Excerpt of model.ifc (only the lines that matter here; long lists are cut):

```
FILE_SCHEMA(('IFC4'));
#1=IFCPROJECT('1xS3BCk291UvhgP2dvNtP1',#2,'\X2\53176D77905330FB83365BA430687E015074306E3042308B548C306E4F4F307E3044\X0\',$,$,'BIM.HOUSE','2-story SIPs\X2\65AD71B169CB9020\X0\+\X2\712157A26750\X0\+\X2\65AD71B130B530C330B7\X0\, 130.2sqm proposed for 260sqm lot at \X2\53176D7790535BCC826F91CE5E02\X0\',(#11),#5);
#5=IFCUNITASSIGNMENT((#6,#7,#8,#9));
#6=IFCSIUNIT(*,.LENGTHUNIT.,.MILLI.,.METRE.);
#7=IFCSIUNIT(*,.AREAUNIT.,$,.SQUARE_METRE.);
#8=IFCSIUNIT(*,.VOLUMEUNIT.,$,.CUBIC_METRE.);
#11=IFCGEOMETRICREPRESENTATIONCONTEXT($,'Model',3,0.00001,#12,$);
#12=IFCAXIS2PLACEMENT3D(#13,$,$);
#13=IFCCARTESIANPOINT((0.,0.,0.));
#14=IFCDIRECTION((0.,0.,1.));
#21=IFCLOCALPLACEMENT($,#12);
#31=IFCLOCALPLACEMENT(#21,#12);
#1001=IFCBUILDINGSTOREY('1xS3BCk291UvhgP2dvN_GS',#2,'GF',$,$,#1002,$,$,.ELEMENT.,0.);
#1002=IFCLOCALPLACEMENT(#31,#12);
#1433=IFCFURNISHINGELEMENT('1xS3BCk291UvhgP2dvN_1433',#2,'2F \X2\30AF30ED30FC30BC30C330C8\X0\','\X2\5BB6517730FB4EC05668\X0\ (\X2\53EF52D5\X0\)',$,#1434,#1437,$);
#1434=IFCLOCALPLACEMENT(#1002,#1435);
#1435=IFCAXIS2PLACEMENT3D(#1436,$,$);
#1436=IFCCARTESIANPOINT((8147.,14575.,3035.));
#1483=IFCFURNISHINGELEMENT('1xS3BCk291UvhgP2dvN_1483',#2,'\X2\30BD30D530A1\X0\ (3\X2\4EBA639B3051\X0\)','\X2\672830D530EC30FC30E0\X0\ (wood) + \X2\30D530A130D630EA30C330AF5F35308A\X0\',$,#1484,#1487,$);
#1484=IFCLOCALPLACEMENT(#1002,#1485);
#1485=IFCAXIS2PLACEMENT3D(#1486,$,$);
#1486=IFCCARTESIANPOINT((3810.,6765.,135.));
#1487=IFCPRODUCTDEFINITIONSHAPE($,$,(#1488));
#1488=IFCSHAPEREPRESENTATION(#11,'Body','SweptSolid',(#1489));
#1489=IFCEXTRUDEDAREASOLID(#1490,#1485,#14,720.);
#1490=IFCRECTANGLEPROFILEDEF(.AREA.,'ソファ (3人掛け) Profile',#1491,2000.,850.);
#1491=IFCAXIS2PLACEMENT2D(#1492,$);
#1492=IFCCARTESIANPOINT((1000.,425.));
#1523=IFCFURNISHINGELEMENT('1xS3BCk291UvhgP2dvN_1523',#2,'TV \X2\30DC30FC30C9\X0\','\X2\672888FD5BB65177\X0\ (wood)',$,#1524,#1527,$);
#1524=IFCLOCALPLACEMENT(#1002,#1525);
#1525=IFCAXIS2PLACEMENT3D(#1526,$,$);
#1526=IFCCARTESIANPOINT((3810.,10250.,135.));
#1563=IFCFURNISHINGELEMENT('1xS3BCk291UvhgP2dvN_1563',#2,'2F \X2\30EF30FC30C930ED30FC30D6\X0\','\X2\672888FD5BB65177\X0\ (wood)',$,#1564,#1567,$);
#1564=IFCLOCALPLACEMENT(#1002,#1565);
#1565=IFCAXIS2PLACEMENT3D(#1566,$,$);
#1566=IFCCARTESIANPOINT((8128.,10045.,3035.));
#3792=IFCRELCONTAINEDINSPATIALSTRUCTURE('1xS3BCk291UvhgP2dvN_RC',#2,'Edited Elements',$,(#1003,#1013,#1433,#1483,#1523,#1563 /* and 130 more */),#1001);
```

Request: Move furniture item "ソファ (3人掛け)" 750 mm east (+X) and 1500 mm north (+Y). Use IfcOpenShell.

```python
import ifcopenshell
import ifcopenshell.api.geometry
import ifcopenshell.util.placement
import ifcopenshell.util.unit

model = ifcopenshell.open("model.ifc")
unit_scale = ifcopenshell.util.unit.calculate_unit_scale(model)

item = model.by_guid("1xS3BCk291UvhgP2dvN_1483")
matrix = ifcopenshell.util.placement.get_local_placement(item.ObjectPlacement)
matrix[0, 3] += 0.75 / unit_scale
matrix[1, 3] += 1.5 / unit_scale
ifcopenshell.api.geometry.edit_object_placement(model, product=item, matrix=matrix, is_si=False)

print(ifcopenshell.util.placement.get_local_placement(item.ObjectPlacement).round(3) + 0.0)

model.write("model_v2.ifc")
```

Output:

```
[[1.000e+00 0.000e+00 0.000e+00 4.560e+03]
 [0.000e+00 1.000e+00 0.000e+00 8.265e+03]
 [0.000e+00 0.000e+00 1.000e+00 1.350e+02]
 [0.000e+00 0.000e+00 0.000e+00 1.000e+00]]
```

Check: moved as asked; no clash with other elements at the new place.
